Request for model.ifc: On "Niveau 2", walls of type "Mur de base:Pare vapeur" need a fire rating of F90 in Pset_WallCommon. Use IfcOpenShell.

First a look at what the model holds.

```python
import ifcopenshell
import ifcopenshell.util.element

model = ifcopenshell.open("model.ifc")
print(model.schema)
storey = next(s for s in model.by_type("IfcBuildingStorey") if s.Name == "Niveau 2")
walls = [e for e in ifcopenshell.util.element.get_decomposition(storey) if e.is_a("IfcWall")]
seen = {}
for e in walls:
    element_type = ifcopenshell.util.element.get_type(e)
    key = (element_type.Name if element_type != e and element_type else None, ifcopenshell.util.element.get_pset(e, "Pset_WallCommon", "FireRating"))
    seen[key] = seen.get(key, 0) + 1
for (name, value), count in sorted(seen.items(), key=str):
    print(count, "x", name, "|", value)
```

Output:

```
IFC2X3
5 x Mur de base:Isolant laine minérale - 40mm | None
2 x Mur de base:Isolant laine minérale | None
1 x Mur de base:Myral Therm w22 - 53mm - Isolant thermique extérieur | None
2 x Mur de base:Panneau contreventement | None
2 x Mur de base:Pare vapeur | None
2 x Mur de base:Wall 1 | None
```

```python
import ifcopenshell
import ifcopenshell.api.pset
import ifcopenshell.util.element

model = ifcopenshell.open("model.ifc")

storey = next(s for s in model.by_type("IfcBuildingStorey") if s.Name == "Niveau 2")
walls = [e for e in ifcopenshell.util.element.get_decomposition(storey) if e.is_a("IfcWall")]

count = 0
for e in walls:
    element_type = ifcopenshell.util.element.get_type(e)
    if element_type in (None, e) or element_type.Name != "Mur de base:Pare vapeur":
        continue
    # add_pset returns the element's existing set when there is one.
    pset = ifcopenshell.api.pset.add_pset(model, product=e, name="Pset_WallCommon")
    ifcopenshell.api.pset.edit_pset(model, pset=pset, properties={"FireRating": "F90"})
    count += 1

print(count, "walls updated")

model.write("model_updated.ifc")
```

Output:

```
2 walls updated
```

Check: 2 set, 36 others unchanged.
